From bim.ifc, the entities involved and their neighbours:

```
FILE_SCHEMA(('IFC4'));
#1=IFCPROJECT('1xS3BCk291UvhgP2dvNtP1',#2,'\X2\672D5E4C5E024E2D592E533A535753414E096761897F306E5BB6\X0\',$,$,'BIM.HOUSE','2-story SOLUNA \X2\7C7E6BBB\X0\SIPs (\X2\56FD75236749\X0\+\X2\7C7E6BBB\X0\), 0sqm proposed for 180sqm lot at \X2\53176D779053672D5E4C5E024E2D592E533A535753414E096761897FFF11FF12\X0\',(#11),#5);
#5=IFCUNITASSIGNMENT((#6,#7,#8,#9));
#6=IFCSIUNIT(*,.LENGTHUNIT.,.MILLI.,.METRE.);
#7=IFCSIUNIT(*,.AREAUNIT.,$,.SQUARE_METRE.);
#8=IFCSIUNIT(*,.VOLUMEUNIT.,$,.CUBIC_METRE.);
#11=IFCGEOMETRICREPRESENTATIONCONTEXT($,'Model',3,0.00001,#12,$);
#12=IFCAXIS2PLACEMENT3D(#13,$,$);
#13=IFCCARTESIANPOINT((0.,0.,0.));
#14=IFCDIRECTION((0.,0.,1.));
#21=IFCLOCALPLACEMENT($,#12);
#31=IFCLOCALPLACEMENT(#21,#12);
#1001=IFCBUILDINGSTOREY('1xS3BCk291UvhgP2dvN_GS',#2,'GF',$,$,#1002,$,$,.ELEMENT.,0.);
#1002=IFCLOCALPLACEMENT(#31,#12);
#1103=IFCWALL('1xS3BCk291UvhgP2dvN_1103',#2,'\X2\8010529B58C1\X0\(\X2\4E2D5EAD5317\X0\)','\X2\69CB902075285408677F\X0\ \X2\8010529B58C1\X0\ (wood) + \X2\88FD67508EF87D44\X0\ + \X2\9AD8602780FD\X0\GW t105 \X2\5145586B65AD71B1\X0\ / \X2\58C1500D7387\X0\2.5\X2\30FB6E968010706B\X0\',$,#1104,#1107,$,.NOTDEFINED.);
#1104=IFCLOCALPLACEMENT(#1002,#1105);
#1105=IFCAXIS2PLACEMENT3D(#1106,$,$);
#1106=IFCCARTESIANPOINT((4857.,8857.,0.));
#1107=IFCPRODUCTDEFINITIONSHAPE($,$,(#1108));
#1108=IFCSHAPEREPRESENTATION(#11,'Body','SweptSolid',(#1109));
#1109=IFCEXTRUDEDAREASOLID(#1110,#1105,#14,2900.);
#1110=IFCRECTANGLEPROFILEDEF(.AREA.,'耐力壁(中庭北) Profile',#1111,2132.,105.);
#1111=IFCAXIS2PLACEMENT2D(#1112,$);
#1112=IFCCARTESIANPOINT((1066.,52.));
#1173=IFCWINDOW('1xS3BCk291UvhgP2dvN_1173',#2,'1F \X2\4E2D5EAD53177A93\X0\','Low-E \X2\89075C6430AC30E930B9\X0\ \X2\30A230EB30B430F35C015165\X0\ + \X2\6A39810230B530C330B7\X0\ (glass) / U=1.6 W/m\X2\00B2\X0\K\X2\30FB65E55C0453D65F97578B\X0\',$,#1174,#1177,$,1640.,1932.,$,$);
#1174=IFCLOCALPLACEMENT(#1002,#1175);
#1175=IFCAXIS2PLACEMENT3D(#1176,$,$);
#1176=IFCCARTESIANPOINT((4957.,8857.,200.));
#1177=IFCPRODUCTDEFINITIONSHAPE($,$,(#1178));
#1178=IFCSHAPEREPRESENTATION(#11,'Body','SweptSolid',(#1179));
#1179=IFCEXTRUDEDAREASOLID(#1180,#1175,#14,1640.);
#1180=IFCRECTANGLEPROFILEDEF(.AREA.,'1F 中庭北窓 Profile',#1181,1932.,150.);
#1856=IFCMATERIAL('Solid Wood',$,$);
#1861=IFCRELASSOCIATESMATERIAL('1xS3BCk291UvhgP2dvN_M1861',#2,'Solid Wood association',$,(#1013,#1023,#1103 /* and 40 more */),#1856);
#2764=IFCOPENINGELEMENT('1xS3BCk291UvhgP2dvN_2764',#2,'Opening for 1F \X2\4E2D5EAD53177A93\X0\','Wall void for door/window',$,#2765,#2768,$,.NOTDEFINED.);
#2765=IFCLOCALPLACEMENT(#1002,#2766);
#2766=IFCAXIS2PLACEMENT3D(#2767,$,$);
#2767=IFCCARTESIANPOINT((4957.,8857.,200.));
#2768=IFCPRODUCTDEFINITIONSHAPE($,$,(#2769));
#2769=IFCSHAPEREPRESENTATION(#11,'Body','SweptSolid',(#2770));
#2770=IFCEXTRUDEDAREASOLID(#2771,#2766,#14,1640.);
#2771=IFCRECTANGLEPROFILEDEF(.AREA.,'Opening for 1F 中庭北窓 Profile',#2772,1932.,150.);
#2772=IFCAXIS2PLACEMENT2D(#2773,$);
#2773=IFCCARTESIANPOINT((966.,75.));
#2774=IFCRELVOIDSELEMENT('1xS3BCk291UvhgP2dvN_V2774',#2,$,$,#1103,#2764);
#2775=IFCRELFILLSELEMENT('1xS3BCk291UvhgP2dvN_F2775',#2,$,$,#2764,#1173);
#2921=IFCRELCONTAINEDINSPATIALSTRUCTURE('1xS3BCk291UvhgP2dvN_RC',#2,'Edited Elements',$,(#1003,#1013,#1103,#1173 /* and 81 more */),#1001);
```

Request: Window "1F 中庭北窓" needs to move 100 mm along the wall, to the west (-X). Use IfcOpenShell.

```python
import ifcopenshell
import ifcopenshell.api.geometry
import ifcopenshell.util.placement

model = ifcopenshell.open("bim.ifc")

window = model.by_guid("1xS3BCk291UvhgP2dvN_1173")
opening = window.FillsVoids[0].RelatingOpeningElement
wall = opening.VoidsElements[0].RelatingBuildingElement

wall_matrix = ifcopenshell.util.placement.get_local_placement(wall.ObjectPlacement)
shift = wall_matrix[:3, 0] * -100.0
before = ifcopenshell.util.placement.get_local_placement(window.ObjectPlacement)[:3, 3].copy()

# The window is not placed relative to its opening, so move both.
for product in (opening, window):
    matrix = ifcopenshell.util.placement.get_local_placement(product.ObjectPlacement)
    matrix[:3, 3] += shift
    ifcopenshell.api.geometry.edit_object_placement(model, product=product, matrix=matrix, is_si=False)

after = ifcopenshell.util.placement.get_local_placement(window.ObjectPlacement)[:3, 3]
print("window moved by", (after - before).round(3) + 0.0)

model.write("bim_rev.ifc")
```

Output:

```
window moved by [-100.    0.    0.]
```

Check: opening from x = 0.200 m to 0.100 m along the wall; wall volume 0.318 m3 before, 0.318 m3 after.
